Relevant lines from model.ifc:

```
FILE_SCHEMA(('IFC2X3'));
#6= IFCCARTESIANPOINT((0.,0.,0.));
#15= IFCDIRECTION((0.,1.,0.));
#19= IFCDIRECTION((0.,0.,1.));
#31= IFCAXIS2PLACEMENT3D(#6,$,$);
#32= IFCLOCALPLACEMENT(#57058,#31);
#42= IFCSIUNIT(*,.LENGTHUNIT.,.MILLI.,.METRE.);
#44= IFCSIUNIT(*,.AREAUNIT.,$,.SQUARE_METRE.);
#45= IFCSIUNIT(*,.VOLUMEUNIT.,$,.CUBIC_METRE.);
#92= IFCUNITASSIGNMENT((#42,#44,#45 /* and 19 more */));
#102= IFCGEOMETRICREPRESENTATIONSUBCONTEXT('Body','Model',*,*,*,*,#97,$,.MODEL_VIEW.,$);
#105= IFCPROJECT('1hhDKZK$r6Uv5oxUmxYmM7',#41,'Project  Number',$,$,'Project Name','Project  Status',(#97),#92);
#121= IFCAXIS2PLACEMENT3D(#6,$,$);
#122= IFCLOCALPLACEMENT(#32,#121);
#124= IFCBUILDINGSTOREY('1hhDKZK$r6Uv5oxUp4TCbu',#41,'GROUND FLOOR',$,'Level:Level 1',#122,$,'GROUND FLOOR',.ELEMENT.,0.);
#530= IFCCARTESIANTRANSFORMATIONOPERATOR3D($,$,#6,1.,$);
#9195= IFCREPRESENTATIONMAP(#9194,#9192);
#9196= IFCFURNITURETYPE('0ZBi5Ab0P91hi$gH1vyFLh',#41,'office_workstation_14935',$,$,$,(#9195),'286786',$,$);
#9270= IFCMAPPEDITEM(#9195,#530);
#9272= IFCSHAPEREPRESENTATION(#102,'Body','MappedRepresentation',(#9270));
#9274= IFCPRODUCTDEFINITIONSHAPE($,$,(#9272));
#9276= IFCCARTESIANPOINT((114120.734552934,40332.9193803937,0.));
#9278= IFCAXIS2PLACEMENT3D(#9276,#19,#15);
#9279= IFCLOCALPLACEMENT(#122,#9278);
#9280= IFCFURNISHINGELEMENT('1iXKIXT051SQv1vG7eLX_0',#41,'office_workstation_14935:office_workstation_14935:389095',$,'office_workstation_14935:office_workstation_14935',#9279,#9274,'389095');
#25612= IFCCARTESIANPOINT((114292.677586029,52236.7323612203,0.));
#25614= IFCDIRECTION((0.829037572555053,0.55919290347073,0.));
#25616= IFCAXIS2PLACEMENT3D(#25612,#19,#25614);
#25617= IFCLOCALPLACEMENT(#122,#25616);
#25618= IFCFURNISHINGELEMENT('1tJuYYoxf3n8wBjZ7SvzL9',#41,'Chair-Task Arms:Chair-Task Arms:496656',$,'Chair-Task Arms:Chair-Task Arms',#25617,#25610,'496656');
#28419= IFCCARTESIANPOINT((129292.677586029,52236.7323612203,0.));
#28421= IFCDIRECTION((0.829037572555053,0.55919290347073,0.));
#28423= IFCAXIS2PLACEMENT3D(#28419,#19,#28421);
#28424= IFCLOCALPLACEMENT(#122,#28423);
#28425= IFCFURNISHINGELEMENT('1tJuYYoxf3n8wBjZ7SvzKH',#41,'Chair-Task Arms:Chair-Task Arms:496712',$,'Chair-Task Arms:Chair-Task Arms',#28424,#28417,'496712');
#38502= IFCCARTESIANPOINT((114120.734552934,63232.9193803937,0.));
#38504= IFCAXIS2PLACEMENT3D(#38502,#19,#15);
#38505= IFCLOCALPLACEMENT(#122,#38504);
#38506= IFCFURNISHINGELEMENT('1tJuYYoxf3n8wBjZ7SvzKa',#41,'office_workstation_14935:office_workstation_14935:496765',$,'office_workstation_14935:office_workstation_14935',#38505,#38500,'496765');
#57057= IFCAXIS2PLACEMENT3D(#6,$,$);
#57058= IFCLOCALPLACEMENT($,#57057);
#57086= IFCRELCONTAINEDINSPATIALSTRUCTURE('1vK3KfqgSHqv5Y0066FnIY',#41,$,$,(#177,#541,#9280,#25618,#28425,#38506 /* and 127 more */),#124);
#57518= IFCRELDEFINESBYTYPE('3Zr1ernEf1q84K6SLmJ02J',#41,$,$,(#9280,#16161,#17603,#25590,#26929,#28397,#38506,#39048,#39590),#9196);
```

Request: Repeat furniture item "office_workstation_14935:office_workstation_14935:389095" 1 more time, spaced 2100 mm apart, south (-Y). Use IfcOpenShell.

```python
import numpy as np
import ifcopenshell
import ifcopenshell.api.geometry
import ifcopenshell.api.root
import ifcopenshell.util.element
import ifcopenshell.util.placement

model = ifcopenshell.open("model.ifc")


def reuse_history(source, copy):
    """copy_class also copies each property set's owner history, people and application; keep the originals."""
    for rel in copy.IsDefinedBy:
        if rel.is_a("IfcRelDefinesByProperties") and (history := rel.RelatingPropertyDefinition.OwnerHistory):
            rel.RelatingPropertyDefinition.OwnerHistory = source.OwnerHistory
            ifcopenshell.util.element.remove_deep2(model, history)


source = model.by_guid("1iXKIXT051SQv1vG7eLX_0")
base = ifcopenshell.util.placement.get_local_placement(source.ObjectPlacement)
step = np.array([0.0, -1.0, 0.0]) * 2100.0

for i in range(1, 2):
    copy = ifcopenshell.api.root.copy_class(model, product=source)
    copy.Representation = ifcopenshell.util.element.copy_deep(
        model, source.Representation, exclude=["IfcGeometricRepresentationContext", "IfcRepresentationMap"]
    )
    copy.Name = "office_workstation_14935:office_workstation_14935"
    copy.Tag = None
    reuse_history(source, copy)
    matrix = base.copy()
    matrix[:3, 3] += i * step
    print("added at", matrix[:3, 3].round(3) + 0.0)
    ifcopenshell.api.geometry.edit_object_placement(model, product=copy, matrix=matrix, is_si=False)

model.write("model_edited.ifc")
```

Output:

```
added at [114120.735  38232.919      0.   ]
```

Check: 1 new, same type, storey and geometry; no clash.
